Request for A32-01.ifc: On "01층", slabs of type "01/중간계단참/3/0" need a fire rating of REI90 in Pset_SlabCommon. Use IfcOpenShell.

First a look at what the model holds.

```python
import ifcopenshell
import ifcopenshell.util.element

model = ifcopenshell.open("A32-01.ifc")
print(model.schema)
storey = next(s for s in model.by_type("IfcBuildingStorey") if s.Name == "01층")
slabs = [e for e in ifcopenshell.util.element.get_decomposition(storey) if e.is_a("IfcSlab")]
seen = {}
for e in slabs:
    element_type = ifcopenshell.util.element.get_type(e)
    key = (element_type.Name if element_type != e and element_type else None, ifcopenshell.util.element.get_pset(e, "Pset_SlabCommon", "FireRating"))
    seen[key] = seen.get(key, 0) + 1
for (name, value), count in sorted(seen.items(), key=str):
    print(count, "x", name, "|", value)
```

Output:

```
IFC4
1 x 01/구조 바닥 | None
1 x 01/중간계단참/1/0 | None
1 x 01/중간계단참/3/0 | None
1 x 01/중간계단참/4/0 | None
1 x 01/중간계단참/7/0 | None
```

```python
import ifcopenshell
import ifcopenshell.api.pset
import ifcopenshell.util.element

model = ifcopenshell.open("A32-01.ifc")

storey = next(s for s in model.by_type("IfcBuildingStorey") if s.Name == "01층")
slabs = [e for e in ifcopenshell.util.element.get_decomposition(storey) if e.is_a("IfcSlab")]

count = 0
for e in slabs:
    element_type = ifcopenshell.util.element.get_type(e)
    if element_type in (None, e) or element_type.Name != "01/중간계단참/3/0":
        continue
    # add_pset returns the element's existing set when there is one.
    pset = ifcopenshell.api.pset.add_pset(model, product=e, name="Pset_SlabCommon")
    ifcopenshell.api.pset.edit_pset(model, pset=pset, properties={"FireRating": "REI90"})
    count += 1

print(count, "slabs updated")

model.write("A32-01_v2.ifc")
```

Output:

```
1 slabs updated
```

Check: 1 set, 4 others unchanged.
